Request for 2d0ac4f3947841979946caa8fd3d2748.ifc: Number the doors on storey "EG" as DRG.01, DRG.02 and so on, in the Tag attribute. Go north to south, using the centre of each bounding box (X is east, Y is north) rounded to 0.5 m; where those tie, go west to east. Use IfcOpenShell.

First a look at what the model holds.

```python
import ifcopenshell
import ifcopenshell.util.element
import ifcopenshell.util.placement

model = ifcopenshell.open("2d0ac4f3947841979946caa8fd3d2748.ifc")
print(model.schema)
storey = next(s for s in model.by_type("IfcBuildingStorey") if s.Name == "EG")
doors = [e for e in ifcopenshell.util.element.get_decomposition(storey) if e.is_a("IfcDoor")]
for e in sorted(doors, key=lambda e: e.id()):
    origin = ifcopenshell.util.placement.get_local_placement(e.ObjectPlacement)[:3, 3]
    print(e.id(), e.Tag, e.Name, origin.round(2) + 0.0, sep=" | ")
```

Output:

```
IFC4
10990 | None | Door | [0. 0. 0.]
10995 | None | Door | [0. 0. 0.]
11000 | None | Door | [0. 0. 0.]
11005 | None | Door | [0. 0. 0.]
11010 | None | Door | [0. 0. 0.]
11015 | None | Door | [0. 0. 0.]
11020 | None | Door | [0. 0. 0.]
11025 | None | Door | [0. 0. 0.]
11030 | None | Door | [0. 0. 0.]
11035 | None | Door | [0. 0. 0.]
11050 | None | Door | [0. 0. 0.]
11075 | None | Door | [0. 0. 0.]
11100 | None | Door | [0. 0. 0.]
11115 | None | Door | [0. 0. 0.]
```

```python
import ifcopenshell
import ifcopenshell.geom
import ifcopenshell.util.element
import ifcopenshell.util.shape

model = ifcopenshell.open("2d0ac4f3947841979946caa8fd3d2748.ifc")
settings = ifcopenshell.geom.settings()
settings.set("use-world-coords", True)


def centre(element):
    shape = ifcopenshell.geom.create_shape(settings, element)
    return ifcopenshell.util.shape.get_bbox_centroid(shape.geometry)


storey = next(s for s in model.by_type("IfcBuildingStorey") if s.Name == "EG")
doors = [e for e in ifcopenshell.util.element.get_decomposition(storey) if e.is_a("IfcDoor")]

# Insertion points can sit at a corner or the storey origin, so sort by the geometry (in metres).
centres = {e: centre(e) for e in doors}
doors.sort(key=lambda e: (-round(centres[e][1] / 0.5), centres[e][0]))

for i, e in enumerate(doors, start=1):
    number = f"DRG.{i:02d}"
    e.Tag = number
    print(e.id(), number)

model.write("2d0ac4f3947841979946caa8fd3d2748-out.ifc")
```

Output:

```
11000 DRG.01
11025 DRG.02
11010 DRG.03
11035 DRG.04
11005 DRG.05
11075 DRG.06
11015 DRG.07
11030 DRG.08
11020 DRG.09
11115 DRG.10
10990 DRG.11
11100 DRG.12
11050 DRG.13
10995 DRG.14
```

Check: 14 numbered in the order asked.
